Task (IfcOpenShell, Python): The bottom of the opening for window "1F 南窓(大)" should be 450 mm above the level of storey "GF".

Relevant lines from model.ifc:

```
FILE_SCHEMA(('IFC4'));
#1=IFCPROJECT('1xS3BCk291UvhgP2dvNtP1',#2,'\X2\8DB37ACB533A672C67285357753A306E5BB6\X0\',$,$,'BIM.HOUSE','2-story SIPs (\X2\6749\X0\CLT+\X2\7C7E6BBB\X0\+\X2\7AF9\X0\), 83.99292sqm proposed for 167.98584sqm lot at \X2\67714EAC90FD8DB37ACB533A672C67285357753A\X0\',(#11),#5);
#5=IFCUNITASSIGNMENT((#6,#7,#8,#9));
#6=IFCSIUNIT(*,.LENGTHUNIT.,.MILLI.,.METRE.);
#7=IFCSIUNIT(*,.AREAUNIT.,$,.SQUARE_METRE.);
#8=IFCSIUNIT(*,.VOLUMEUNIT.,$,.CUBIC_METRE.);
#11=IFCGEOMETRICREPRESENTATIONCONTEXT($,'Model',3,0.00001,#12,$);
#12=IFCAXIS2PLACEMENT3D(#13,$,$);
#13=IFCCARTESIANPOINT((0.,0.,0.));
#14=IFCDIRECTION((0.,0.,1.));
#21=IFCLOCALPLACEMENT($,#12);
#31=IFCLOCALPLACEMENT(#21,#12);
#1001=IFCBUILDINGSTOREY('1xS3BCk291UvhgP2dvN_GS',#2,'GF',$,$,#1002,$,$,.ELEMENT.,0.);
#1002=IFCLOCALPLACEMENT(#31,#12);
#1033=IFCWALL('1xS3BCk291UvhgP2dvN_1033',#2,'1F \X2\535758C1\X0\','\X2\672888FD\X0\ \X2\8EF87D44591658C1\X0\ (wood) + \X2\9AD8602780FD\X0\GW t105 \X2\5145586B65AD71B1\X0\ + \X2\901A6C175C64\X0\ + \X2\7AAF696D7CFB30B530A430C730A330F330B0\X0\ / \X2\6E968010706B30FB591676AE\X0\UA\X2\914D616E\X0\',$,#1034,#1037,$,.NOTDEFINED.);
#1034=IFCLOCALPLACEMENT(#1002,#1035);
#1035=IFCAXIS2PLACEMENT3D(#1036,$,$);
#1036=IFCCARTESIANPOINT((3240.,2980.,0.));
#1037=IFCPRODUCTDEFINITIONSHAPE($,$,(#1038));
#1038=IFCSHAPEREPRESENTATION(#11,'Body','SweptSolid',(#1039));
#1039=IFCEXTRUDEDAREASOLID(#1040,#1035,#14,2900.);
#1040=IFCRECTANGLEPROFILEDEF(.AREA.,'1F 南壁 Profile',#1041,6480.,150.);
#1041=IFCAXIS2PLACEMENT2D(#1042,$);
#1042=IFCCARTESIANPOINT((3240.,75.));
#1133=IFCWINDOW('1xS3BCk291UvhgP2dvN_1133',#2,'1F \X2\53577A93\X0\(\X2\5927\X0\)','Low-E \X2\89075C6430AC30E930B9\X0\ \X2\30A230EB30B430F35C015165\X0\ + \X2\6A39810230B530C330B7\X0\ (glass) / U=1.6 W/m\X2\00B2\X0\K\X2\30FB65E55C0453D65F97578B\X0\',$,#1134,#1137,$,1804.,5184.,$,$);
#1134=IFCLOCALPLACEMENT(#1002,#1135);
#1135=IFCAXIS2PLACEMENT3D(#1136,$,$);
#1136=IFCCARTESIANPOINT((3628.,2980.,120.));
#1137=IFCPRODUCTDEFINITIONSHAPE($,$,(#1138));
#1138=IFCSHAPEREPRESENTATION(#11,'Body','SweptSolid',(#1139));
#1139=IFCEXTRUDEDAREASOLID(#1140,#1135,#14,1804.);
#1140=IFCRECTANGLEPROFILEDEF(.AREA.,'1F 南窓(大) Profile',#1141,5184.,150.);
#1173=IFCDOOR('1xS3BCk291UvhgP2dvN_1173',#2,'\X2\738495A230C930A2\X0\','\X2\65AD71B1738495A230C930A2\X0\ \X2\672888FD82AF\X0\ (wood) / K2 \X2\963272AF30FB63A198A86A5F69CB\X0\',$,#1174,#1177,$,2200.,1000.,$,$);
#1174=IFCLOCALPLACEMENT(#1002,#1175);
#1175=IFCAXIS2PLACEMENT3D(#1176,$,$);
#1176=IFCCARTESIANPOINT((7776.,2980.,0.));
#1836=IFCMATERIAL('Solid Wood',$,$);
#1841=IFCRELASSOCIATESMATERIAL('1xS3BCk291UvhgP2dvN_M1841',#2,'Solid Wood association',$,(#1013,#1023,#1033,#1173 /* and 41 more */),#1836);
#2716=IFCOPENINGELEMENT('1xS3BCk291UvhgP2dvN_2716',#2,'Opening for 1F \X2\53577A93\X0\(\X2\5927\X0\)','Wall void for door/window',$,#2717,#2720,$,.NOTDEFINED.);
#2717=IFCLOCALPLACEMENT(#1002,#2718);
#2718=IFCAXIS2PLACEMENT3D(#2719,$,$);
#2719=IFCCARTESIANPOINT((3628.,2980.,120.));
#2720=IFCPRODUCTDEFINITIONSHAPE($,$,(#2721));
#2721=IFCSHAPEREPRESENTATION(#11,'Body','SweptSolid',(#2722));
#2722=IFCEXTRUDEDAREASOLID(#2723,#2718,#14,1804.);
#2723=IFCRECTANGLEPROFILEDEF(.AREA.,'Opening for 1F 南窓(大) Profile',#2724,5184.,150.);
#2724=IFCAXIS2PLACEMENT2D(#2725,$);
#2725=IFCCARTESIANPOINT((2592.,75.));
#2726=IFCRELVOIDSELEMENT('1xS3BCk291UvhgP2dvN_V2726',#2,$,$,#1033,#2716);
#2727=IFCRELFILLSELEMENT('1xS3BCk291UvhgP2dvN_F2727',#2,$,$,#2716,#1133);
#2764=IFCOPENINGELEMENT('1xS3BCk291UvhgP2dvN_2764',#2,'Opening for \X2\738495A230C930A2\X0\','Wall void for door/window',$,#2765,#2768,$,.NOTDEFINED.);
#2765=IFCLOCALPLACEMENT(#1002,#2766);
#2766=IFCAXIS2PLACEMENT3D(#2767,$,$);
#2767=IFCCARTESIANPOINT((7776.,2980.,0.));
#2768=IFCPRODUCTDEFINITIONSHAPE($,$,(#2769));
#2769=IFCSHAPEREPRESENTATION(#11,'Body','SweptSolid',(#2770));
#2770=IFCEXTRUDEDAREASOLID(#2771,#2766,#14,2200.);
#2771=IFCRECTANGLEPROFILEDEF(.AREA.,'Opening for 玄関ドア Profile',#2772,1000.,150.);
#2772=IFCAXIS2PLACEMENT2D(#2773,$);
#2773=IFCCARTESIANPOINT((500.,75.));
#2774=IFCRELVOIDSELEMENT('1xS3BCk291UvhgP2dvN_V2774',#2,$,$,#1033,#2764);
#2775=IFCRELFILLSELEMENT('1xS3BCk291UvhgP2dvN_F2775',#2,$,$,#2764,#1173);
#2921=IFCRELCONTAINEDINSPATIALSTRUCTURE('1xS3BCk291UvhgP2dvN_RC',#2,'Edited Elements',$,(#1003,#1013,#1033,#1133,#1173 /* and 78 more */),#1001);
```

```python
import numpy as np
import ifcopenshell
import ifcopenshell.api.geometry
import ifcopenshell.geom
import ifcopenshell.util.element
import ifcopenshell.util.placement
import ifcopenshell.util.shape
import ifcopenshell.util.unit

model = ifcopenshell.open("model.ifc")
unit_scale = ifcopenshell.util.unit.calculate_unit_scale(model)

window = model.by_guid("1xS3BCk291UvhgP2dvN_1133")
opening = window.FillsVoids[0].RelatingOpeningElement
storey = ifcopenshell.util.element.get_container(window, ifc_class="IfcBuildingStorey")
level = ifcopenshell.util.placement.get_local_placement(storey.ObjectPlacement)[2, 3]

# The opening's origin need not be at the sill, so measure its lowest point.
shape = ifcopenshell.geom.create_shape(ifcopenshell.geom.settings(), opening)
bottom = ifcopenshell.util.shape.get_shape_bottom_elevation(shape, shape.geometry) / unit_scale
dz = level + 0.45 / unit_scale - bottom

shift = np.array([0.0, 0.0, dz])
# The window is not placed relative to its opening, so move both.
for product in (opening, window):
    matrix = ifcopenshell.util.placement.get_local_placement(product.ObjectPlacement)
    matrix[:3, 3] += shift
    ifcopenshell.api.geometry.edit_object_placement(model, product=product, matrix=matrix, is_si=False)

print(f"moved by {dz * unit_scale:+.3f} m")

model.write("model_edited.ifc")
```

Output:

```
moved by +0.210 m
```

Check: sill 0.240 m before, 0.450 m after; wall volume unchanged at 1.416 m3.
